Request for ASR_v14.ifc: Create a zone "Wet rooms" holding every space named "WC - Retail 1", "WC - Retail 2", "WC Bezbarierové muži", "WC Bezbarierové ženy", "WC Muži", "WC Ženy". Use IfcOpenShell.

First a look at what the model holds.

```python
import ifcopenshell

model = ifcopenshell.open("ASR_v14.ifc")
print(model.schema)
seen = {}
for space in model.by_type("IfcSpace"):
    seen[space.LongName] = seen.get(space.LongName, 0) + 1
for name, count in sorted(seen.items(), key=str):
    print(count, "x", name)
print("zones:", [z.Name for z in model.by_type("IfcZone")][:20])
```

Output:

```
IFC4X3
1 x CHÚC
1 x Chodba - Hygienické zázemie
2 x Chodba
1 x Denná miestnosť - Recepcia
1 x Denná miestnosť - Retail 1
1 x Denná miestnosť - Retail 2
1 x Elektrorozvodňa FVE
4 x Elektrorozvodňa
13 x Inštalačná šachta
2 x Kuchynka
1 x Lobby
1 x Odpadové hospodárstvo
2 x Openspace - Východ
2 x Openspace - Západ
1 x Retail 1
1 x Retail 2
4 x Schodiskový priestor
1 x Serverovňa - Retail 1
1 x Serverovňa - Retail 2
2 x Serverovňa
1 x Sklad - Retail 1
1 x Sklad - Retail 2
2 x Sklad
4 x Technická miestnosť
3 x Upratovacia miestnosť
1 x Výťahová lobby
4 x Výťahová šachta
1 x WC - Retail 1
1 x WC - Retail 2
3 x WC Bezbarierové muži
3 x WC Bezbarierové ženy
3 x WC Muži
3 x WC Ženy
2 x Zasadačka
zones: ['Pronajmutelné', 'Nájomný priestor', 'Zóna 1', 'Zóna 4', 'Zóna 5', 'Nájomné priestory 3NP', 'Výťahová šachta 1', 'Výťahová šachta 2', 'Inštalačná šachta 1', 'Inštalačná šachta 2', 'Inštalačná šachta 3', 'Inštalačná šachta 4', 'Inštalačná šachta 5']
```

```python
import ifcopenshell
import ifcopenshell.api.group
import ifcopenshell.api.root

model = ifcopenshell.open("ASR_v14.ifc")

names = {"WC - Retail 1", "WC - Retail 2", "WC Bezbarierové muži", "WC Bezbarierové ženy", "WC Muži", "WC Ženy"}
spaces = [s for s in model.by_type("IfcSpace") if s.LongName in names]

zone = ifcopenshell.api.root.create_entity(model, ifc_class="IfcZone", name="Wet rooms")
ifcopenshell.api.group.assign_group(model, products=spaces, group=zone)
print(len(spaces), "spaces in", zone.Name)

model.write("ASR_v14_v2.ifc")
```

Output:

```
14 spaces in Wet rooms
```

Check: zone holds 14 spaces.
